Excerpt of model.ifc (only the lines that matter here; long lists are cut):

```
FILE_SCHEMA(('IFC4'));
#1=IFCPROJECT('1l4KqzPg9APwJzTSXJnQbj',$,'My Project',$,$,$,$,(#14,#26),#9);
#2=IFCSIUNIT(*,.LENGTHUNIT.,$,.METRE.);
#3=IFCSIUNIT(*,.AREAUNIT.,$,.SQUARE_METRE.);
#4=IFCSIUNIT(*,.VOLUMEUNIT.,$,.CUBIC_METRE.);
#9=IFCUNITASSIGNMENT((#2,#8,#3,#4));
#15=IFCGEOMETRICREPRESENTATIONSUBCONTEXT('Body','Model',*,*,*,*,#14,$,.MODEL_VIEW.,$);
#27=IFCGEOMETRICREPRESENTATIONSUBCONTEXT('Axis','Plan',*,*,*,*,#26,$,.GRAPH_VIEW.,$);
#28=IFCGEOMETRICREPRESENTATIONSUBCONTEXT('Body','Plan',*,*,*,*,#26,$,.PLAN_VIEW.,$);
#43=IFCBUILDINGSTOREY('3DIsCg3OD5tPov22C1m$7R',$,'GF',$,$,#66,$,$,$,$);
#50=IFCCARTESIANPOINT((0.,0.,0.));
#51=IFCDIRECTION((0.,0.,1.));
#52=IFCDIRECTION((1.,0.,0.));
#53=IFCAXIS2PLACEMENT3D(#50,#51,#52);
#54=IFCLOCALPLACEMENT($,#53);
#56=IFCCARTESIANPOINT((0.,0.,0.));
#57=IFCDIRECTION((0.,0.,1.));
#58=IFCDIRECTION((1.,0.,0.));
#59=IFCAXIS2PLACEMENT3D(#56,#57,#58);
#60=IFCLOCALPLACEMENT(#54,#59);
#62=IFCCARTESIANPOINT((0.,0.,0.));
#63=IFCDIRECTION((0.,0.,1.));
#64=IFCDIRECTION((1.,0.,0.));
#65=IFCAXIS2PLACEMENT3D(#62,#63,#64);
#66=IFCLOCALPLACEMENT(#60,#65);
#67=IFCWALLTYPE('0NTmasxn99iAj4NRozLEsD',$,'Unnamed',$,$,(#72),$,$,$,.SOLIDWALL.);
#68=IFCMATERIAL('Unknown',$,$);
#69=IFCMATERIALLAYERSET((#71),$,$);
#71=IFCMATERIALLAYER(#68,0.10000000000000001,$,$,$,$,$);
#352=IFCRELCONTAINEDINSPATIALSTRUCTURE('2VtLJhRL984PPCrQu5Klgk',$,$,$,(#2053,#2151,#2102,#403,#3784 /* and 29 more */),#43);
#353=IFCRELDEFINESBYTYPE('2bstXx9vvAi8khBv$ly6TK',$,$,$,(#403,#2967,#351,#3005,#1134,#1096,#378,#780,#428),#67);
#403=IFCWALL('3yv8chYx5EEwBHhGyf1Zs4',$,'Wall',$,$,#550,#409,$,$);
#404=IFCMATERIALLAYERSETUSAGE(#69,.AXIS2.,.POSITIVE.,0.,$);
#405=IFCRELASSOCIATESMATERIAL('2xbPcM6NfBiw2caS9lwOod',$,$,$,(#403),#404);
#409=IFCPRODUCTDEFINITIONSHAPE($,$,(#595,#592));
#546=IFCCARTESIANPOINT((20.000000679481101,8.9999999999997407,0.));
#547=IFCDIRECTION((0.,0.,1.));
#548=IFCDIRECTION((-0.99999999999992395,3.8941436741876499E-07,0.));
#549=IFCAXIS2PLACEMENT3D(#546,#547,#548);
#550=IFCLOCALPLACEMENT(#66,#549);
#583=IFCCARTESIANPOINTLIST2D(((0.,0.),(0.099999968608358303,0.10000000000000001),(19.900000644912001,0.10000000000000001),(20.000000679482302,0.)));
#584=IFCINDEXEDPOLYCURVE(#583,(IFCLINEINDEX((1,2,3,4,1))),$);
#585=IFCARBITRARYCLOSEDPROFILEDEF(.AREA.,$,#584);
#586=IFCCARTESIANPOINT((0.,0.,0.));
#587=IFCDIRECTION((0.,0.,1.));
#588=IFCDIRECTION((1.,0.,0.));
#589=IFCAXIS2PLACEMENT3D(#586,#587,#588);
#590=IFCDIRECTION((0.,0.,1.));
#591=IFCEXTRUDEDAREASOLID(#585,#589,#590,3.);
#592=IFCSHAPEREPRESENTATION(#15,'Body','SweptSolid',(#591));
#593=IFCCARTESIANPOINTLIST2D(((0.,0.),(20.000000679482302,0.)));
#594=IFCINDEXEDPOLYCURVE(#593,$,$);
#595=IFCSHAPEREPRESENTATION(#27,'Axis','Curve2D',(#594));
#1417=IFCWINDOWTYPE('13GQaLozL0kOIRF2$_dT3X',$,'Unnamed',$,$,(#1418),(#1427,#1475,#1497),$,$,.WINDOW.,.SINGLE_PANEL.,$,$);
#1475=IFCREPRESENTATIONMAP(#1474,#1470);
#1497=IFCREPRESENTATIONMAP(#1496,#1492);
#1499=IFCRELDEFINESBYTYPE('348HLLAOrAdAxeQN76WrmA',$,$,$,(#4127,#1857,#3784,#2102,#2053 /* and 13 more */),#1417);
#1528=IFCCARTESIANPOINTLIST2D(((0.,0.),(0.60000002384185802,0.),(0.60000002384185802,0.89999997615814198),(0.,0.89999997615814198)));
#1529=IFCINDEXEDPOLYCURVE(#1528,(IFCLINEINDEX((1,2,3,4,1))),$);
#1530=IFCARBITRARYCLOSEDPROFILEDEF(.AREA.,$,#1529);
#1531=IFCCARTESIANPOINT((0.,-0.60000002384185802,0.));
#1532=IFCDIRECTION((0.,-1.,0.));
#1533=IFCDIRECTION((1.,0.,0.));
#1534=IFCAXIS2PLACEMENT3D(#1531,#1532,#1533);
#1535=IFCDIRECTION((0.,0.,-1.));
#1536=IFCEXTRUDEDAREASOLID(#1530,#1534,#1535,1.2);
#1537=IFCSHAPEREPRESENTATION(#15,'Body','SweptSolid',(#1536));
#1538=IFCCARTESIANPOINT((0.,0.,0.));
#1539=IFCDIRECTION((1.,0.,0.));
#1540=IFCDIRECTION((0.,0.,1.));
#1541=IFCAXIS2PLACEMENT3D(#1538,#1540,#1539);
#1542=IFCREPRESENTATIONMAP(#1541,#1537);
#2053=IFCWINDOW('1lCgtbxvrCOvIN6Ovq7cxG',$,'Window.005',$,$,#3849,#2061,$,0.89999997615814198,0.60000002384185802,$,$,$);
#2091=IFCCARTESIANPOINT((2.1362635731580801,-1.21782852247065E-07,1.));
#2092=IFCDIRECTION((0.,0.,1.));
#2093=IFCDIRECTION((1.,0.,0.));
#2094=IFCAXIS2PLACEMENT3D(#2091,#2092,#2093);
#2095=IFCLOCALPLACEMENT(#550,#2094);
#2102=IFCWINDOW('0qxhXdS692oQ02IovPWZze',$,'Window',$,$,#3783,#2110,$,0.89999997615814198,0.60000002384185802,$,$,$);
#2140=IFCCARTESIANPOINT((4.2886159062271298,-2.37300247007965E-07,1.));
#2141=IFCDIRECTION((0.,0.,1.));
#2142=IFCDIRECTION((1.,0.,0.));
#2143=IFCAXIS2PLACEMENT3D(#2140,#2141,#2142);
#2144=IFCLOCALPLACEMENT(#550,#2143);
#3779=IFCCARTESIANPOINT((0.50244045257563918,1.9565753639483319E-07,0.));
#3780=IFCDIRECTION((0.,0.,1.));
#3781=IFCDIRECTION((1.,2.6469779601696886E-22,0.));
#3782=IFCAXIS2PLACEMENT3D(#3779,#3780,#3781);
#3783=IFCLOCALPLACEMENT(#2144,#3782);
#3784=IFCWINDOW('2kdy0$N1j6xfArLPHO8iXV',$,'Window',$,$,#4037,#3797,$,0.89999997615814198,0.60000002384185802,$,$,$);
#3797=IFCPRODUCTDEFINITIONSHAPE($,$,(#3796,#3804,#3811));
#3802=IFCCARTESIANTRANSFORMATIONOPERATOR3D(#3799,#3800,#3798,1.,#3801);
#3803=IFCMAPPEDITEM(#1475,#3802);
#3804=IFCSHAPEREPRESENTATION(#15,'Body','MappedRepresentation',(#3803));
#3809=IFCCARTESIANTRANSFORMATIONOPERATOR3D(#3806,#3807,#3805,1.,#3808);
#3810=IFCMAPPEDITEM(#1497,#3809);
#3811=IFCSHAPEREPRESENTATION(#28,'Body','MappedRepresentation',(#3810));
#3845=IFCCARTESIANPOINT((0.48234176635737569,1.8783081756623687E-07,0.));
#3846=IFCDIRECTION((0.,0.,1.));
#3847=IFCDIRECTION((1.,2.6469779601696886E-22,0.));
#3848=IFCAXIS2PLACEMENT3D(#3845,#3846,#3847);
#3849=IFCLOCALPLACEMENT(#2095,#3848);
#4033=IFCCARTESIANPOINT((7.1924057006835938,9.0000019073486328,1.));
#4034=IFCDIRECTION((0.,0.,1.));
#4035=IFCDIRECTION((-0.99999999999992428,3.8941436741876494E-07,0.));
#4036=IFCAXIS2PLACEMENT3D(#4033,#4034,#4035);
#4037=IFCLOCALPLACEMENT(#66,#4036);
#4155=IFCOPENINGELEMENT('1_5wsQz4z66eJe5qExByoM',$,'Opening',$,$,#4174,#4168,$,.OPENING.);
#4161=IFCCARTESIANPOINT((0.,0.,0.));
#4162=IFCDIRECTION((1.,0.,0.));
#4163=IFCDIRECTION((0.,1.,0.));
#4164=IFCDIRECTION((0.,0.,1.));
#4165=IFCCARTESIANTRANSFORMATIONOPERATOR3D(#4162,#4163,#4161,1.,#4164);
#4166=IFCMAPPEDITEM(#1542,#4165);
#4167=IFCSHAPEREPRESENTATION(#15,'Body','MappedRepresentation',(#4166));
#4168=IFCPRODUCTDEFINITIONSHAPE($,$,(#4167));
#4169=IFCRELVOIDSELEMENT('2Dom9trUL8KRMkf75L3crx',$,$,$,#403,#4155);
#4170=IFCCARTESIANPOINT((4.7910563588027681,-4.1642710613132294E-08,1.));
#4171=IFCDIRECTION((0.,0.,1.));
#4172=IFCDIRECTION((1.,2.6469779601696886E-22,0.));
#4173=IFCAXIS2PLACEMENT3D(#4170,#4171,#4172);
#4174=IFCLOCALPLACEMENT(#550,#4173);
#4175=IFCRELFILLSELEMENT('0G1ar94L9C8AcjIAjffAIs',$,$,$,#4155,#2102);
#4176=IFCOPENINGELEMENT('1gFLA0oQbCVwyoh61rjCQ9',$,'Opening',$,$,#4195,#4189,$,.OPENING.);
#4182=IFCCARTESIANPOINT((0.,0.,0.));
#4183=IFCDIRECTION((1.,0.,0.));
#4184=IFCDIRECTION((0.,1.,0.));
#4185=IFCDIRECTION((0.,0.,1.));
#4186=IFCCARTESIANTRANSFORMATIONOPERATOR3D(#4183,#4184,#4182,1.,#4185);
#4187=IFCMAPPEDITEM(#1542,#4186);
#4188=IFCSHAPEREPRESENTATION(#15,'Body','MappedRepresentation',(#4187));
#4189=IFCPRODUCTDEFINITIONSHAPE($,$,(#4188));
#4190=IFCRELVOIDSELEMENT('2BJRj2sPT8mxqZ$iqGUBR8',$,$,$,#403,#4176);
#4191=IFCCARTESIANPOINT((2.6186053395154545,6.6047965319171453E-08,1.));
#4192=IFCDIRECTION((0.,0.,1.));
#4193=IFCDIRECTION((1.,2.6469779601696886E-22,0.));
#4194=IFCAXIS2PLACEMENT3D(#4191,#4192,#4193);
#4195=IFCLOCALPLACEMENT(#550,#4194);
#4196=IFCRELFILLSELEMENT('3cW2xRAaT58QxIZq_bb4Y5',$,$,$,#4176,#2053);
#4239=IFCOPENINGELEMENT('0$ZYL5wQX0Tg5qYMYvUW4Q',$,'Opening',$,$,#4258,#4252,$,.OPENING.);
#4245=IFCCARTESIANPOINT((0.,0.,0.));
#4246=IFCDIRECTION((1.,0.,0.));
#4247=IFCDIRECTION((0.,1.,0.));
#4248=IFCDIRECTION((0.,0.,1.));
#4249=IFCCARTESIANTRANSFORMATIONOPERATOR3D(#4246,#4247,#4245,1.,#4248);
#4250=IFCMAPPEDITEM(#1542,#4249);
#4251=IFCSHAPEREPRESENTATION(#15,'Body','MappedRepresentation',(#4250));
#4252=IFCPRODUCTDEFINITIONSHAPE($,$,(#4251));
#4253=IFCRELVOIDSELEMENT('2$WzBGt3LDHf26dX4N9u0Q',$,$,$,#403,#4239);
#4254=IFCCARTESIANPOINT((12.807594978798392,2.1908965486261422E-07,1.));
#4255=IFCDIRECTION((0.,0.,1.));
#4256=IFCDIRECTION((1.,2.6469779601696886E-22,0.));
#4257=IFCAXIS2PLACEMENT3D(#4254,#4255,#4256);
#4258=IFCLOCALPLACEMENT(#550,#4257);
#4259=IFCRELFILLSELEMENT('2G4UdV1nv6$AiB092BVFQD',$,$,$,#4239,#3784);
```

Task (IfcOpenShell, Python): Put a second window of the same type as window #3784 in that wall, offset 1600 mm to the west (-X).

```python
import ifcopenshell
import ifcopenshell.api.feature
import ifcopenshell.api.geometry
import ifcopenshell.api.root
import ifcopenshell.geom
import ifcopenshell.util.element
import ifcopenshell.util.placement
import ifcopenshell.util.shape

model = ifcopenshell.open("model.ifc")
settings = ifcopenshell.geom.settings()


def volume(element):
    """Net volume in cubic metres, openings subtracted."""
    shape = ifcopenshell.geom.create_shape(settings, element)
    return ifcopenshell.util.shape.get_volume(shape.geometry)


window = model.by_id(3784)
opening = window.FillsVoids[0].RelatingOpeningElement
wall = opening.VoidsElements[0].RelatingBuildingElement
before = volume(wall)
shift = ifcopenshell.util.placement.get_local_placement(wall.ObjectPlacement)[:3, 0] * 1.6

# copy_class copies the void relationship, type, container and properties, but no geometry.
new_opening = ifcopenshell.api.root.copy_class(model, product=opening)
new_opening.Representation = ifcopenshell.util.element.copy_deep(
    model, opening.Representation, exclude=["IfcGeometricRepresentationContext", "IfcRepresentationMap"]
)
new_window = ifcopenshell.api.root.copy_class(model, product=window)
new_window.Representation = ifcopenshell.util.element.copy_deep(
    model, window.Representation, exclude=["IfcGeometricRepresentationContext", "IfcRepresentationMap"]
)
ifcopenshell.api.feature.add_filling(model, opening=new_opening, element=new_window)

for old, new in ((opening, new_opening), (window, new_window)):
    matrix = ifcopenshell.util.placement.get_local_placement(old.ObjectPlacement)
    matrix[:3, 3] += shift
    ifcopenshell.api.geometry.edit_object_placement(model, product=new, matrix=matrix, is_si=False)

after = volume(wall)

print(f"wall volume {before:.3f} -> {after:.3f} m3")

model.write("model_updated.ifc")
```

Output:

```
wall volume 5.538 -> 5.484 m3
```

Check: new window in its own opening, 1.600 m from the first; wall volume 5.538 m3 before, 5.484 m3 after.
